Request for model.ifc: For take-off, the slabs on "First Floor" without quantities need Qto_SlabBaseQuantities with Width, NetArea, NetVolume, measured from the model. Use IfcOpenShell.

First a look at what the model holds.

```python
import ifcopenshell
import ifcopenshell.util.element
import ifcopenshell.util.unit

model = ifcopenshell.open("model.ifc")
print(model.schema)
for unit_type in ("LENGTHUNIT", "AREAUNIT", "VOLUMEUNIT"):
    print(unit_type, ifcopenshell.util.unit.calculate_unit_scale(model, unit_type))
storey = next(s for s in model.by_type("IfcBuildingStorey") if s.Name == "First Floor")
slabs = [e for e in ifcopenshell.util.element.get_decomposition(storey) if e.is_a("IfcSlab")]
for e in sorted(slabs, key=lambda e: e.id()):
    print(e.id(), e.is_a(), e.Name, list(ifcopenshell.util.element.get_psets(e, qtos_only=True)), sep=" | ")
```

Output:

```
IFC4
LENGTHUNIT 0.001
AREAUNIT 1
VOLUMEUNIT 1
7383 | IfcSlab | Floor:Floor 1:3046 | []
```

```python
import ifcopenshell
import ifcopenshell.api.pset
import ifcopenshell.geom
import ifcopenshell.util.element
import ifcopenshell.util.shape
import ifcopenshell.util.unit

model = ifcopenshell.open("model.ifc")
unit_scale = ifcopenshell.util.unit.calculate_unit_scale(model)
area_scale = ifcopenshell.util.unit.calculate_unit_scale(model, "AREAUNIT")
volume_scale = ifcopenshell.util.unit.calculate_unit_scale(model, "VOLUMEUNIT")
settings = ifcopenshell.geom.settings()

storey = next(s for s in model.by_type("IfcBuildingStorey") if s.Name == "First Floor")
slabs = [e for e in ifcopenshell.util.element.get_decomposition(storey) if e.is_a("IfcSlab")]

for e in sorted(slabs, key=lambda e: e.id()):
    if ifcopenshell.util.element.get_psets(e, qtos_only=True, should_inherit=False):
        continue
    # Geometry comes back in metres, in the element's own axes.
    shape = ifcopenshell.geom.create_shape(settings, e)
    values = {
        "Width": ifcopenshell.util.shape.get_z(shape.geometry) / unit_scale,
        "NetArea": ifcopenshell.util.shape.get_footprint_area(shape.geometry) / area_scale,
        "NetVolume": ifcopenshell.util.shape.get_volume(shape.geometry) / volume_scale,
    }
    qto = ifcopenshell.api.pset.add_qto(model, product=e, name="Qto_SlabBaseQuantities")
    ifcopenshell.api.pset.edit_qto(model, qto=qto, properties=values)
    print(e.id(), {k: round(v, 3) for k, v in values.items()})

model.write("model_edited.ifc")
```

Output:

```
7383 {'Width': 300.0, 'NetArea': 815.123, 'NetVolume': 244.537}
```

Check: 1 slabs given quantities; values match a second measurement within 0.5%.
